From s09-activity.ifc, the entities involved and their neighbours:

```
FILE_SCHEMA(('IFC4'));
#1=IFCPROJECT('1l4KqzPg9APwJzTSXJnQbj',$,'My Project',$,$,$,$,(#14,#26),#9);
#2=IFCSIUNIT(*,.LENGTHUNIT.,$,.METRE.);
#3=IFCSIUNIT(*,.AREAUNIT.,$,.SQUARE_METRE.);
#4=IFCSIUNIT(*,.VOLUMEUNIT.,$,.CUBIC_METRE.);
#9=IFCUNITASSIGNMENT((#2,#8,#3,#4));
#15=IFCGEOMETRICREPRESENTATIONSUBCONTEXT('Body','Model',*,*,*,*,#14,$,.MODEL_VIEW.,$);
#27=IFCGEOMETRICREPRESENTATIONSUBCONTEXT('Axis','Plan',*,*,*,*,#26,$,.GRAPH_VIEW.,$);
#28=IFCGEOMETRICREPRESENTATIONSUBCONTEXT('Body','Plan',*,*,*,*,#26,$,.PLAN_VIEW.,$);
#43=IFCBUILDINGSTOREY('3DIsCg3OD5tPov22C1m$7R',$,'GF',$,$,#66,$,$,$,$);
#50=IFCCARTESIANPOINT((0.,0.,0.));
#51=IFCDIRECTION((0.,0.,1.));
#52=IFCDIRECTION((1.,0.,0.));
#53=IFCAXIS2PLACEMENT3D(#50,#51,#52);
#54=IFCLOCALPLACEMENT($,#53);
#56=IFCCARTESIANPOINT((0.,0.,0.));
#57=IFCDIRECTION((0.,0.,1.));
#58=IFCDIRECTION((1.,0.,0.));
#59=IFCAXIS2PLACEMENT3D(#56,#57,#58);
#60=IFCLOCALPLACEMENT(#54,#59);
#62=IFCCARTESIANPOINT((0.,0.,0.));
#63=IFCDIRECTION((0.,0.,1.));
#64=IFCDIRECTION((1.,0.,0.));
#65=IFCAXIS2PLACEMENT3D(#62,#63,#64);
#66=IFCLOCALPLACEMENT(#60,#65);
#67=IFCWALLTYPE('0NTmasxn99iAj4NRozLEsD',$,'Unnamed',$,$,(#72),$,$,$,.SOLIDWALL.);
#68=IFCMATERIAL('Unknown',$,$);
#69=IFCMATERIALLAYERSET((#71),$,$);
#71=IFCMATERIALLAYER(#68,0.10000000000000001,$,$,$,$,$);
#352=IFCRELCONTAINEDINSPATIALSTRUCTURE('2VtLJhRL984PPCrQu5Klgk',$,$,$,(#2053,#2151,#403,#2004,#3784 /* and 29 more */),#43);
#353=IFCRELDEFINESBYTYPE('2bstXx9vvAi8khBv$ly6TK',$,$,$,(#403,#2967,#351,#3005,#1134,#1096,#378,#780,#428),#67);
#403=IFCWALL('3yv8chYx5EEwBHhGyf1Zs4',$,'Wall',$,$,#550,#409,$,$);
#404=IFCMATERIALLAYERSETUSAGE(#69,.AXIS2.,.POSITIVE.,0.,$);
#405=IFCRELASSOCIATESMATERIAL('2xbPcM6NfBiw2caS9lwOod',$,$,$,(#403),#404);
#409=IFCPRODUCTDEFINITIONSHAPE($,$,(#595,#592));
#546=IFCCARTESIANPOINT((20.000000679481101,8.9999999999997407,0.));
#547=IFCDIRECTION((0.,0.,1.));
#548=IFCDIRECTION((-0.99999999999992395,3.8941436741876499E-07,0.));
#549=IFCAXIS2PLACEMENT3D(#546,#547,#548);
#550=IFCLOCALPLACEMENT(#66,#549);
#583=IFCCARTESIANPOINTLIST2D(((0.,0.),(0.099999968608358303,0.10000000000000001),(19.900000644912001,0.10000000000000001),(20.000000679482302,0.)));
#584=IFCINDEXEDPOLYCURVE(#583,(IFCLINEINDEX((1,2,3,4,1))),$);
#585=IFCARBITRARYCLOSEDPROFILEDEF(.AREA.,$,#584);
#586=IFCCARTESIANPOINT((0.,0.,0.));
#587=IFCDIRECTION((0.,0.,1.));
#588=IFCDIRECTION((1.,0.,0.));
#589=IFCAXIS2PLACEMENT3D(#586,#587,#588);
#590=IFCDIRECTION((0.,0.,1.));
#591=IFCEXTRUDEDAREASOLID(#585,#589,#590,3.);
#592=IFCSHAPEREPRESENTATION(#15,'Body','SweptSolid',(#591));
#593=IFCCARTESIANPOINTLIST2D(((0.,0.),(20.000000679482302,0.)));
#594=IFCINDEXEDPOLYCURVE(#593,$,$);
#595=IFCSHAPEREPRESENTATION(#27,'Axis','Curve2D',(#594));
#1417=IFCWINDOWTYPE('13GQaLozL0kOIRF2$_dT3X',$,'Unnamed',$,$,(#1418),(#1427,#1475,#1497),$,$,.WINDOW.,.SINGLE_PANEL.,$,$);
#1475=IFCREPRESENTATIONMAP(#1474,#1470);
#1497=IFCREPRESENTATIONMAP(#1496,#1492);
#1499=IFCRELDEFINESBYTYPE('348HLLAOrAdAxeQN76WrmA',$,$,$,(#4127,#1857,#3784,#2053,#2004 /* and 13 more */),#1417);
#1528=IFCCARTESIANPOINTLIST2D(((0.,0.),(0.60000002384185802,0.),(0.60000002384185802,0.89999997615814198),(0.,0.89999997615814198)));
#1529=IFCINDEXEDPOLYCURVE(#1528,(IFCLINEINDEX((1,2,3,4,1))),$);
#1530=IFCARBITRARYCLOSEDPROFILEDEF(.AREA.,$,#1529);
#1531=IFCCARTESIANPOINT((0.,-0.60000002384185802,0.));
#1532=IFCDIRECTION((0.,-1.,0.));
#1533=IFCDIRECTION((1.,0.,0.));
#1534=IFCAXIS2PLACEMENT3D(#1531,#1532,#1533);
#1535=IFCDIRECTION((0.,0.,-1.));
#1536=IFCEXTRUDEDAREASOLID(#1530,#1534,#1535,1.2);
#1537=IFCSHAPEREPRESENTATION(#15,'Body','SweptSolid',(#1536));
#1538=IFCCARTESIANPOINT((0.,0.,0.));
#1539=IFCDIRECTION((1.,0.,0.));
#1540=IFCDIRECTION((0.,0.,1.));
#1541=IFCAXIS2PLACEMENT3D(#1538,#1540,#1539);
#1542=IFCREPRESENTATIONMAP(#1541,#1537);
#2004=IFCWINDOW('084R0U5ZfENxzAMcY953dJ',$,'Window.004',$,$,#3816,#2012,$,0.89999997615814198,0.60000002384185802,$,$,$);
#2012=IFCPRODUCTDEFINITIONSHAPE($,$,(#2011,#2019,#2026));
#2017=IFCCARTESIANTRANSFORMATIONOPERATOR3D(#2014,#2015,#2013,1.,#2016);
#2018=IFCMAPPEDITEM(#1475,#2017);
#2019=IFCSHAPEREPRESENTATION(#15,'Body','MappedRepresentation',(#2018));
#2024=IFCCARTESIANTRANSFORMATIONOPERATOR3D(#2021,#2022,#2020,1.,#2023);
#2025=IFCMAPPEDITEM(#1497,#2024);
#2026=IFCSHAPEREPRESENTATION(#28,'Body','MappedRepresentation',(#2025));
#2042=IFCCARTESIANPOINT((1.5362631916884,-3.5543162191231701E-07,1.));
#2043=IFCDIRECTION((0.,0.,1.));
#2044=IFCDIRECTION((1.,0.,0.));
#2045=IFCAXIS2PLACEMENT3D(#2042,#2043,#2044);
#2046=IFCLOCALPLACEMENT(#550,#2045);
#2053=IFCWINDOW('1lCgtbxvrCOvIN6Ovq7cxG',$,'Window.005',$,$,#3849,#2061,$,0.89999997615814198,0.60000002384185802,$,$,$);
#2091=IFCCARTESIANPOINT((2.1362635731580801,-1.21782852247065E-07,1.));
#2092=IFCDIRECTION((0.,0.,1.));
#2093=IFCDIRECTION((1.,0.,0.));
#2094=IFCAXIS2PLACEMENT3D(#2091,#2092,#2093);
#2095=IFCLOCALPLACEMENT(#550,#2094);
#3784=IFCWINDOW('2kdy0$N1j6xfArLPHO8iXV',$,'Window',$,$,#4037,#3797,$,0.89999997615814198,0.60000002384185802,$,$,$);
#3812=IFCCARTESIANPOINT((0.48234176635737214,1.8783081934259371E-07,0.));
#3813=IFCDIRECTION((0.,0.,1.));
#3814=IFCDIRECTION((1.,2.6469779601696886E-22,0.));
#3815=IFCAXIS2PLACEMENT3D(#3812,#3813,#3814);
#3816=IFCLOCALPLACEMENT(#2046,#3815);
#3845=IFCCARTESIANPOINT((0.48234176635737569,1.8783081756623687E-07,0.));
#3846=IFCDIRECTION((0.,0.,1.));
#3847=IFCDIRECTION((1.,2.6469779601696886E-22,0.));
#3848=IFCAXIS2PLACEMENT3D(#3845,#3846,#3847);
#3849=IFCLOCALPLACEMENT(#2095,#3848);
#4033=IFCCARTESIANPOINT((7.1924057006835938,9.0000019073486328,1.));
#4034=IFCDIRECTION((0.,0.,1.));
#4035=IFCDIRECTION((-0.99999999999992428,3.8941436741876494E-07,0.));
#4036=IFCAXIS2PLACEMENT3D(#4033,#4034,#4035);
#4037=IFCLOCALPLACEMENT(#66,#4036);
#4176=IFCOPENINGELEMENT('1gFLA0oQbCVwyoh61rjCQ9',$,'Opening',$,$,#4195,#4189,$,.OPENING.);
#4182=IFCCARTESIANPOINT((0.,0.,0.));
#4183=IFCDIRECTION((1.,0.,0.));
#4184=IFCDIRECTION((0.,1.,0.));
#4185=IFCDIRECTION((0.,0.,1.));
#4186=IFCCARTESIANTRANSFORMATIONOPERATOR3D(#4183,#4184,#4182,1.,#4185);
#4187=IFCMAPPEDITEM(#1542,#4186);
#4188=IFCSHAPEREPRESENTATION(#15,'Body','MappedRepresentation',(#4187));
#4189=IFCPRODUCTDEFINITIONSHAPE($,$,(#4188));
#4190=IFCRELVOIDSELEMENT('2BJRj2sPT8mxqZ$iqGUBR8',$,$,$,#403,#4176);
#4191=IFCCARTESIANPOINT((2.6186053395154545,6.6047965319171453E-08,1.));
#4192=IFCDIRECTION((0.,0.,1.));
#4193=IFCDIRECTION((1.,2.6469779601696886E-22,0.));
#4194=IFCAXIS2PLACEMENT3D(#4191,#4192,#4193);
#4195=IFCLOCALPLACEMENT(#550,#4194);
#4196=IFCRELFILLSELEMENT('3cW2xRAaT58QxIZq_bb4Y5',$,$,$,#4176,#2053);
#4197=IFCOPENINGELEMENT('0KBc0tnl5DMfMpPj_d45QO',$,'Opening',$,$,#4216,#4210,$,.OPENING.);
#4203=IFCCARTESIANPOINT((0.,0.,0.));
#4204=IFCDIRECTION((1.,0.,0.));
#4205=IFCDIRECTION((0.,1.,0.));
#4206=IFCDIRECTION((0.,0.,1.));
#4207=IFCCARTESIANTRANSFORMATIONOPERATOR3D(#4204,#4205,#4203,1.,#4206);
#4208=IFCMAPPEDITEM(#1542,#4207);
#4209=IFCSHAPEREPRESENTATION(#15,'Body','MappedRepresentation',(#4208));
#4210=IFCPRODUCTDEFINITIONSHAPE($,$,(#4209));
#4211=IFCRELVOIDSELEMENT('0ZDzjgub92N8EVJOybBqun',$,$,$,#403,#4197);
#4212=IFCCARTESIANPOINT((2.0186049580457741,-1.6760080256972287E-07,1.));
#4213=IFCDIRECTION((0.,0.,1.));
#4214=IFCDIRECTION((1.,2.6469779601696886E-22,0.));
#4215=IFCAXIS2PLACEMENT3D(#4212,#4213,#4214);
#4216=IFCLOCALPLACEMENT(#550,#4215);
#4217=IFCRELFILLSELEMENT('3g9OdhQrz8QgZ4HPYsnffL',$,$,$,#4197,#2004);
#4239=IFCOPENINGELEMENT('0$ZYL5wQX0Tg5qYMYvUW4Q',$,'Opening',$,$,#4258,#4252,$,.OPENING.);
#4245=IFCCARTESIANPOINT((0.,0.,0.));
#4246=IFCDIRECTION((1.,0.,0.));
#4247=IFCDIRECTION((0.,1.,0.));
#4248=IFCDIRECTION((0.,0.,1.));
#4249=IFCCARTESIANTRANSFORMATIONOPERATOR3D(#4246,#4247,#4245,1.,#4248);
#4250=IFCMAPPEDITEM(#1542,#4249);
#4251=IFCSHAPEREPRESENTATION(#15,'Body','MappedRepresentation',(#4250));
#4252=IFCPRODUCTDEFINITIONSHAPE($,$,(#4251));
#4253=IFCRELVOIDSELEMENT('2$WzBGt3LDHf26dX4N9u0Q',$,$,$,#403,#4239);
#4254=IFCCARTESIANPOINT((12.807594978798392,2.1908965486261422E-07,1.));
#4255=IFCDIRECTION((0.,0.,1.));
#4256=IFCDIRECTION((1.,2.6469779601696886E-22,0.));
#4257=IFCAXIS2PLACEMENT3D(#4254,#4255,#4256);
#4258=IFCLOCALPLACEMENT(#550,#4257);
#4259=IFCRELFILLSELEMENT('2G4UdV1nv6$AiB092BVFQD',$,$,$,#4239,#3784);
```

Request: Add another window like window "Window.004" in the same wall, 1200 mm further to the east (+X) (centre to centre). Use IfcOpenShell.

```python
import ifcopenshell
import ifcopenshell.api.feature
import ifcopenshell.api.geometry
import ifcopenshell.api.root
import ifcopenshell.geom
import ifcopenshell.util.element
import ifcopenshell.util.placement
import ifcopenshell.util.shape
import ifcopenshell.util.unit

model = ifcopenshell.open("s09-activity.ifc")
unit_scale = ifcopenshell.util.unit.calculate_unit_scale(model)
settings = ifcopenshell.geom.settings()


def volume(element):
    """Net volume in cubic metres, openings subtracted."""
    shape = ifcopenshell.geom.create_shape(settings, element)
    return ifcopenshell.util.shape.get_volume(shape.geometry)


window = model.by_guid("084R0U5ZfENxzAMcY953dJ")
opening = window.FillsVoids[0].RelatingOpeningElement
wall = opening.VoidsElements[0].RelatingBuildingElement
before = volume(wall)
shift = ifcopenshell.util.placement.get_local_placement(wall.ObjectPlacement)[:3, 0] * -1.2 / unit_scale

# copy_class copies the void relationship, type, container and properties, but no geometry.
new_opening = ifcopenshell.api.root.copy_class(model, product=opening)
new_opening.Representation = ifcopenshell.util.element.copy_deep(
    model, opening.Representation, exclude=["IfcGeometricRepresentationContext", "IfcRepresentationMap"]
)
new_window = ifcopenshell.api.root.copy_class(model, product=window)
new_window.Representation = ifcopenshell.util.element.copy_deep(
    model, window.Representation, exclude=["IfcGeometricRepresentationContext", "IfcRepresentationMap"]
)
ifcopenshell.api.feature.add_filling(model, opening=new_opening, element=new_window)

for old, new in ((opening, new_opening), (window, new_window)):
    matrix = ifcopenshell.util.placement.get_local_placement(old.ObjectPlacement)
    matrix[:3, 3] += shift
    ifcopenshell.api.geometry.edit_object_placement(model, product=new, matrix=matrix, is_si=False)

after = volume(wall)

print(f"wall volume {before:.3f} -> {after:.3f} m3")

model.write("s09-activity_rev.ifc")
```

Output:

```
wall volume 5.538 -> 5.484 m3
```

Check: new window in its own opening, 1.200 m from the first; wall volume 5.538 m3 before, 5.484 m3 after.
